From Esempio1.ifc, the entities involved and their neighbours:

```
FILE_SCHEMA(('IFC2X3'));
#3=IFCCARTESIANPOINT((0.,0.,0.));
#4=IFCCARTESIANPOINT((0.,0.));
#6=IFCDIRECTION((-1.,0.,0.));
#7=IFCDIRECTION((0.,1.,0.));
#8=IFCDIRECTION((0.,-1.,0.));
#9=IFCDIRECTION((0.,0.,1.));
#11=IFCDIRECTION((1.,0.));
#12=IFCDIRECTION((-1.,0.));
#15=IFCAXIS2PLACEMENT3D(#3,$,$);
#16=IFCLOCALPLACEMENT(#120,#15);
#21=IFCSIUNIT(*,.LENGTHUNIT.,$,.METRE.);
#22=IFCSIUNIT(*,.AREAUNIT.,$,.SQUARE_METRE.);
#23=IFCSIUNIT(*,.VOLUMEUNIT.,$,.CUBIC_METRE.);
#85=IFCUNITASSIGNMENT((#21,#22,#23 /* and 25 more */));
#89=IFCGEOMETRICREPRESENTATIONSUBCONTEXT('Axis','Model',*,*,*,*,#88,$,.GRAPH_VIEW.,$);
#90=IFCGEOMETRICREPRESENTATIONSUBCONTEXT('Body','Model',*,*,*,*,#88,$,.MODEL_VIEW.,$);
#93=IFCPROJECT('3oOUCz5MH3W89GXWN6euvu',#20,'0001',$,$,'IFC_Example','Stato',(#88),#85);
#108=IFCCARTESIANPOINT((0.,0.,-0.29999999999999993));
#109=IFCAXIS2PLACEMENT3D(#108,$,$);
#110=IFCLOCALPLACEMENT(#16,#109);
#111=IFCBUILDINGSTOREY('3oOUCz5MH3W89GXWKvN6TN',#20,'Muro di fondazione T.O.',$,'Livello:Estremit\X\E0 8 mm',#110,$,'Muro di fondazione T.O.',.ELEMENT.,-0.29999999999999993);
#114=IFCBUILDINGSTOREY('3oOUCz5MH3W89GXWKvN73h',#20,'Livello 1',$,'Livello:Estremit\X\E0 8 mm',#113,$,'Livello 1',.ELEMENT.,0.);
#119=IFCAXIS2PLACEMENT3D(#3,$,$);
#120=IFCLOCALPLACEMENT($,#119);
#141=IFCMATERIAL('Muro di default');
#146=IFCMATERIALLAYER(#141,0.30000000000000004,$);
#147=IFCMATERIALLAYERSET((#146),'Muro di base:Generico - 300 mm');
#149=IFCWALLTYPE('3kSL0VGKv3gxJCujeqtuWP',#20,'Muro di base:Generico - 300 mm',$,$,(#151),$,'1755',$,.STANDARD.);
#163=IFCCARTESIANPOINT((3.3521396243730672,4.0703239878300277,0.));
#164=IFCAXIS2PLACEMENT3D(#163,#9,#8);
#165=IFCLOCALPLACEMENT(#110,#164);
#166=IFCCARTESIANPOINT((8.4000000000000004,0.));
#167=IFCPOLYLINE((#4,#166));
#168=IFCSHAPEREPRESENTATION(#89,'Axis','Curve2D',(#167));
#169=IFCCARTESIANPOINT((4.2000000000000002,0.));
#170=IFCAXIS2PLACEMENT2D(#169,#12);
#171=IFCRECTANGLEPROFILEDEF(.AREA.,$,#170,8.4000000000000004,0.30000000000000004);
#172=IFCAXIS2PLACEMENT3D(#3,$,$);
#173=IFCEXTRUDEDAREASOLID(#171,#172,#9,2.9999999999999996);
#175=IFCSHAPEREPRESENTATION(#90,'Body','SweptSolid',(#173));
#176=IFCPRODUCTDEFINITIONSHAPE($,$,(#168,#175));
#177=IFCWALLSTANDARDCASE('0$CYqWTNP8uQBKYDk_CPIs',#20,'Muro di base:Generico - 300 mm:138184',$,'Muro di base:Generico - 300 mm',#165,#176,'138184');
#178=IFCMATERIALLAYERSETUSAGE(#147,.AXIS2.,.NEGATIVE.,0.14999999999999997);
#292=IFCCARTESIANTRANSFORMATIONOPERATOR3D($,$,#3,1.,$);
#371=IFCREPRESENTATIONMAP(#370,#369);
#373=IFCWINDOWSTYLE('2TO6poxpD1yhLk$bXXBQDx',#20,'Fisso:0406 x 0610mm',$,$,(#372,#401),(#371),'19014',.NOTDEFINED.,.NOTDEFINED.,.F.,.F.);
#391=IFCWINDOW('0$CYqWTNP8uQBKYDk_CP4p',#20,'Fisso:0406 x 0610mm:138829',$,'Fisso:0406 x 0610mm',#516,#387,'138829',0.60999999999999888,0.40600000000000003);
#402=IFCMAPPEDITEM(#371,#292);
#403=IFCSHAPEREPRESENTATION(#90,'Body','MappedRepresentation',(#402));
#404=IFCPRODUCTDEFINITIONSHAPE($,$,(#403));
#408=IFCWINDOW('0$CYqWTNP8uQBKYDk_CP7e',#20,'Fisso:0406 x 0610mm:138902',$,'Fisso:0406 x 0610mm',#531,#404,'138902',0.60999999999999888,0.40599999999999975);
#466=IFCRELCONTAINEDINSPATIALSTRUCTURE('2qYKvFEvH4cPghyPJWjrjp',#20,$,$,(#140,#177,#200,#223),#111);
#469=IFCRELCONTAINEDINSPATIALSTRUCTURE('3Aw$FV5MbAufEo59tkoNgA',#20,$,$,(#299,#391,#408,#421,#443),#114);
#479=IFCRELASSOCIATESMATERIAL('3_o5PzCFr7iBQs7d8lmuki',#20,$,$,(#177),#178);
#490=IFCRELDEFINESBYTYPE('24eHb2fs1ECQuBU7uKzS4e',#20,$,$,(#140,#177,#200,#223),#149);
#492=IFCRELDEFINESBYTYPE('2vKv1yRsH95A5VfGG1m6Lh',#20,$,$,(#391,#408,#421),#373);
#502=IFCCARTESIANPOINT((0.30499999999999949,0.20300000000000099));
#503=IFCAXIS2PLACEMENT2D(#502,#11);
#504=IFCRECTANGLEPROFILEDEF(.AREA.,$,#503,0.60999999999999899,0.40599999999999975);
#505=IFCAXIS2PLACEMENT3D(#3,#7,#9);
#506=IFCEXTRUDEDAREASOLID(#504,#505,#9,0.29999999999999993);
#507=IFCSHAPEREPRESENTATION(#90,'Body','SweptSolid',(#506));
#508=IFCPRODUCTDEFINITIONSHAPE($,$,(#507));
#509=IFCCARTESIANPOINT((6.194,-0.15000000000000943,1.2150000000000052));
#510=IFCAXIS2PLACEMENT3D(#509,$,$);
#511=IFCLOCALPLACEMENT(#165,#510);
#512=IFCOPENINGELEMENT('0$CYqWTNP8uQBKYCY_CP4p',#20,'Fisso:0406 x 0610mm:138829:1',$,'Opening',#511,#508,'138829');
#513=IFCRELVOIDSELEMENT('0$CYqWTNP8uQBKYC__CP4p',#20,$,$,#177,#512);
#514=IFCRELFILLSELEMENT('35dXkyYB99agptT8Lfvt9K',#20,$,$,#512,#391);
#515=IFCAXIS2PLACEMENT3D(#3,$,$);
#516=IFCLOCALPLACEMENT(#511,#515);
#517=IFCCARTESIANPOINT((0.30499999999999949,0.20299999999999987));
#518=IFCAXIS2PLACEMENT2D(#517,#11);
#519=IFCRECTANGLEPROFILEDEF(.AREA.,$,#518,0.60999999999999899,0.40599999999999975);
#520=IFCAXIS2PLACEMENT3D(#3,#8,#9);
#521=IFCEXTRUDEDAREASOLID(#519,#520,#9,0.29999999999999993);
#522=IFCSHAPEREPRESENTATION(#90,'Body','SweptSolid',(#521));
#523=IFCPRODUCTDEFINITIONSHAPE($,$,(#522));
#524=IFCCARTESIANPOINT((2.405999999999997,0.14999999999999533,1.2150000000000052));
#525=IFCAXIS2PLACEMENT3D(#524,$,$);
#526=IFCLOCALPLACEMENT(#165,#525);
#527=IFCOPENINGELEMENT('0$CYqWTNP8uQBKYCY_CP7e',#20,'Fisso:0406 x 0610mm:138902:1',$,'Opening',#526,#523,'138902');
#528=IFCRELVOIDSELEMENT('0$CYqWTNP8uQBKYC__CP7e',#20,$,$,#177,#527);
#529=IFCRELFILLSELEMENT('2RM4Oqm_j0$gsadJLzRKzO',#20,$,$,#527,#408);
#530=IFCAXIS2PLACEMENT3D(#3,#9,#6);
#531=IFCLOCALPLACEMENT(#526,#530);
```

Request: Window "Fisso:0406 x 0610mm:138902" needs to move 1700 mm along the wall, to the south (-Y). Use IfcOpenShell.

```python
import ifcopenshell
import ifcopenshell.api.geometry
import ifcopenshell.util.placement
import ifcopenshell.util.unit

model = ifcopenshell.open("Esempio1.ifc")
unit_scale = ifcopenshell.util.unit.calculate_unit_scale(model)

window = model.by_guid("0$CYqWTNP8uQBKYDk_CP7e")
opening = window.FillsVoids[0].RelatingOpeningElement
wall = opening.VoidsElements[0].RelatingBuildingElement

wall_matrix = ifcopenshell.util.placement.get_local_placement(wall.ObjectPlacement)
shift = wall_matrix[:3, 0] * 1.7 / unit_scale
before = ifcopenshell.util.placement.get_local_placement(window.ObjectPlacement)[:3, 3].copy()

# The window is placed relative to its opening, so it follows when the opening moves.
matrix = ifcopenshell.util.placement.get_local_placement(opening.ObjectPlacement)
matrix[:3, 3] += shift
ifcopenshell.api.geometry.edit_object_placement(
    model, product=opening, matrix=matrix, is_si=False, should_transform_children=True
)

after = ifcopenshell.util.placement.get_local_placement(window.ObjectPlacement)[:3, 3]
print("window moved by", (after - before).round(3) + 0.0)

model.write("Esempio1-out.ifc")
```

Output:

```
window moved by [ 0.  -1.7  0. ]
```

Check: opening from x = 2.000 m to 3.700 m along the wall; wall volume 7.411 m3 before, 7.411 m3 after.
